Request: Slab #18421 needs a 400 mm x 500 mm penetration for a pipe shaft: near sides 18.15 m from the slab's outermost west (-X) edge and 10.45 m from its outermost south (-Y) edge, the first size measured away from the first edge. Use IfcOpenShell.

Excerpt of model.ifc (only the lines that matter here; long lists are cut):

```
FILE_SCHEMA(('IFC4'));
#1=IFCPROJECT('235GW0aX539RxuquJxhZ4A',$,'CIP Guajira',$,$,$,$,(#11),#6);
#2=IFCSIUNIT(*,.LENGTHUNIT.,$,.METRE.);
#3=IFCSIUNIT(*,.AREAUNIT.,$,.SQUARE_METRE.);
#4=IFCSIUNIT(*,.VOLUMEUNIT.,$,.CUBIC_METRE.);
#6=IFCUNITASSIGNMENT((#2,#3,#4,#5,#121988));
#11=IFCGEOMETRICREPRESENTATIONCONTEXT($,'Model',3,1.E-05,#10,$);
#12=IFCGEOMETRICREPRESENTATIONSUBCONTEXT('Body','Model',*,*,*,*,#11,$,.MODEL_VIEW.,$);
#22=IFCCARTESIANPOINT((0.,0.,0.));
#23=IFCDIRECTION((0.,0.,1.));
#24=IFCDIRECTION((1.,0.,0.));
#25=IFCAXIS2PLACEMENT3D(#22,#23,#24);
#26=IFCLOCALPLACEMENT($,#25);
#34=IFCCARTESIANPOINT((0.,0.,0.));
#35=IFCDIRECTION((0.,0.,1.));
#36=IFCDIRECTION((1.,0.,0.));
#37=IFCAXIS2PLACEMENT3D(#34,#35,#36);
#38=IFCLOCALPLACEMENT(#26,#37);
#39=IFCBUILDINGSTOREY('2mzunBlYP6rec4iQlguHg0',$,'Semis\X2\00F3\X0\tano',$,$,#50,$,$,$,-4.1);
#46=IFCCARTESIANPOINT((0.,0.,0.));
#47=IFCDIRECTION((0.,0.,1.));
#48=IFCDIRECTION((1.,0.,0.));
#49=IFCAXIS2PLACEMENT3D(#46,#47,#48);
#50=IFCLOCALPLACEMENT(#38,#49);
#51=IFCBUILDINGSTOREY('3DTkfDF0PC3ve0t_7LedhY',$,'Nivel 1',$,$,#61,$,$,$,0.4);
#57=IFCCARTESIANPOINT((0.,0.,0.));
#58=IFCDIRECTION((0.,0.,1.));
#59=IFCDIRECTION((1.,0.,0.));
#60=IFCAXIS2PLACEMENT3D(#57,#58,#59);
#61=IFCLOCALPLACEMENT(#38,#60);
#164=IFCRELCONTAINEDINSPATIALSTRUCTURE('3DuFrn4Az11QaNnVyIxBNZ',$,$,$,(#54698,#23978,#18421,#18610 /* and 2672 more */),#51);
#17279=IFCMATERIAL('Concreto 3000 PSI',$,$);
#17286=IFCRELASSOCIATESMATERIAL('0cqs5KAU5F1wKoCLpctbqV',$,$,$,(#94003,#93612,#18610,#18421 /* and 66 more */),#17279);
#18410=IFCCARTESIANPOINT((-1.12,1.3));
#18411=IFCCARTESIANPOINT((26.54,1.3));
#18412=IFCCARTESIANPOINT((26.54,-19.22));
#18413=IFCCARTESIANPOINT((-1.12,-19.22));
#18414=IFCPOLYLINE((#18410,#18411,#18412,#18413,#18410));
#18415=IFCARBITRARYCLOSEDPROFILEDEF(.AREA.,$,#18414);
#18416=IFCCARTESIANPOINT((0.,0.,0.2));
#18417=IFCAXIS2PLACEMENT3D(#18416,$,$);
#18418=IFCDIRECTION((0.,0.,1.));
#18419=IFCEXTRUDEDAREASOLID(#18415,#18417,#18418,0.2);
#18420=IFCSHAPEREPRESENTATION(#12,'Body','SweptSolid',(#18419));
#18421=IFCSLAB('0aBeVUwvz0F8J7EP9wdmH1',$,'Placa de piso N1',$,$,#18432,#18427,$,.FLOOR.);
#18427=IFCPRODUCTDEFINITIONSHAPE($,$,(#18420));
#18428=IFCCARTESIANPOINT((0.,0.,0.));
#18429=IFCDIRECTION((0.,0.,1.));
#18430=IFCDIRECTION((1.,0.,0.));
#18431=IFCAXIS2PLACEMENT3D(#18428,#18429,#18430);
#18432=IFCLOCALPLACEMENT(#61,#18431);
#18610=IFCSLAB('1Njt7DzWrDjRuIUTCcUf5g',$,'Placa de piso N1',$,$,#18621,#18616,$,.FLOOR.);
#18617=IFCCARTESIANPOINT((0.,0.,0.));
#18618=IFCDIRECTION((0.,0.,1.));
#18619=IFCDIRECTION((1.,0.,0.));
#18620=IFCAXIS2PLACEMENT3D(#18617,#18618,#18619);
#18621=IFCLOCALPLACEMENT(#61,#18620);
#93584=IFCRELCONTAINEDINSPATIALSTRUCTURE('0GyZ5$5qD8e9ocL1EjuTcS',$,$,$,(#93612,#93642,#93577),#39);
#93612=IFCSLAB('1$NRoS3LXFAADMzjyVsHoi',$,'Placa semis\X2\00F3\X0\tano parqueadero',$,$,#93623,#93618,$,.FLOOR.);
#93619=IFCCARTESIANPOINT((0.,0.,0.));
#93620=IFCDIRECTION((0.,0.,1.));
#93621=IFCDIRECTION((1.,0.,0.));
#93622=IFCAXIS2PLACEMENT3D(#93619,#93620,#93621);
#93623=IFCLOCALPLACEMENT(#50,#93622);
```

```python
import numpy as np
import ifcopenshell
import ifcopenshell.api.feature
import ifcopenshell.api.geometry
import ifcopenshell.api.root
import ifcopenshell.geom
import ifcopenshell.util.placement
import ifcopenshell.util.representation
import ifcopenshell.util.shape
import ifcopenshell.util.unit

model = ifcopenshell.open("model.ifc")
unit_scale = ifcopenshell.util.unit.calculate_unit_scale(model)
settings = ifcopenshell.geom.settings()


def volume(element):
    """Net volume in cubic metres, openings subtracted."""
    shape = ifcopenshell.geom.create_shape(settings, element)
    return ifcopenshell.util.shape.get_volume(shape.geometry)


slab = model.by_guid("0aBeVUwvz0F8J7EP9wdmH1")
before = volume(slab)

# Extent in the slab's own axes, in metres. The edges named are its -X and -Y sides.
slab_shape = ifcopenshell.geom.create_shape(settings, slab)
vertices = ifcopenshell.util.shape.get_vertices(slab_shape.geometry)
x_min, y_min, bottom = vertices.min(axis=0)
top = vertices[:, 2].max()

opening = ifcopenshell.api.root.create_entity(model, ifc_class="IfcOpeningElement", name="Pipe shaft opening", predefined_type="OPENING")
context = ifcopenshell.util.representation.get_context(model, "Model", "Body", "MODEL_VIEW")
width, depth = 0.4, 0.5
outline = [(0.0, 0.0), (width, 0.0), (width, depth), (0.0, depth), (0.0, 0.0)]
# Overshoot both faces by 50 mm so the cut is clean.
shape = ifcopenshell.api.geometry.add_slab_representation(
    model, context=context, depth=top - bottom + 0.1, polyline=outline
)
ifcopenshell.api.geometry.assign_representation(model, product=opening, representation=shape)

matrix = ifcopenshell.util.placement.get_local_placement(slab.ObjectPlacement)
matrix[:, 3] = matrix @ np.append(np.array([x_min + 18.15, y_min + 10.45, bottom - 0.05]) / unit_scale, 1.0)
ifcopenshell.api.geometry.edit_object_placement(model, product=opening, matrix=matrix, is_si=False)
ifcopenshell.api.feature.add_feature(model, feature=opening, element=slab)

after = volume(slab)

print(f"slab volume {before:.3f} -> {after:.3f} m3")

model.write("model_edited.ifc")
```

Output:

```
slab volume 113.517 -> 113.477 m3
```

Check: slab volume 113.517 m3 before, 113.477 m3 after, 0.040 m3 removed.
